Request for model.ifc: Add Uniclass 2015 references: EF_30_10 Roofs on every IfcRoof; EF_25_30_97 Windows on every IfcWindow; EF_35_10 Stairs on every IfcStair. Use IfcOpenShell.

First a look at what the model holds.

```python
import ifcopenshell

model = ifcopenshell.open("model.ifc")
print(model.schema)
print("classifications:", [c.Name for c in model.by_type("IfcClassification")])
for ifc_class in ("IfcDoor", "IfcRoof", "IfcStair", "IfcWall", "IfcWindow"):
    print(ifc_class, len(model.by_type(ifc_class)))
```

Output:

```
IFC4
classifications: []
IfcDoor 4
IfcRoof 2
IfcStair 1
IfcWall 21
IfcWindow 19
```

```python
import ifcopenshell
import ifcopenshell.api.classification

model = ifcopenshell.open("model.ifc")

system = ifcopenshell.api.classification.add_classification(model, classification="Uniclass 2015")

codes = {
    "IfcRoof": ("EF_30_10", "Roofs"),
    "IfcWindow": ("EF_25_30_97", "Windows"),
    "IfcStair": ("EF_35_10", "Stairs"),
}
for ifc_class, (code, name) in codes.items():
    products = model.by_type(ifc_class)
    ifcopenshell.api.classification.add_reference(
        model, products=products, classification=system, identification=code, name=name
    )
    print(code, len(products))

model.write("model_updated.ifc")
```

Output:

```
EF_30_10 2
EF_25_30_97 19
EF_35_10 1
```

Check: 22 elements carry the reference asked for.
